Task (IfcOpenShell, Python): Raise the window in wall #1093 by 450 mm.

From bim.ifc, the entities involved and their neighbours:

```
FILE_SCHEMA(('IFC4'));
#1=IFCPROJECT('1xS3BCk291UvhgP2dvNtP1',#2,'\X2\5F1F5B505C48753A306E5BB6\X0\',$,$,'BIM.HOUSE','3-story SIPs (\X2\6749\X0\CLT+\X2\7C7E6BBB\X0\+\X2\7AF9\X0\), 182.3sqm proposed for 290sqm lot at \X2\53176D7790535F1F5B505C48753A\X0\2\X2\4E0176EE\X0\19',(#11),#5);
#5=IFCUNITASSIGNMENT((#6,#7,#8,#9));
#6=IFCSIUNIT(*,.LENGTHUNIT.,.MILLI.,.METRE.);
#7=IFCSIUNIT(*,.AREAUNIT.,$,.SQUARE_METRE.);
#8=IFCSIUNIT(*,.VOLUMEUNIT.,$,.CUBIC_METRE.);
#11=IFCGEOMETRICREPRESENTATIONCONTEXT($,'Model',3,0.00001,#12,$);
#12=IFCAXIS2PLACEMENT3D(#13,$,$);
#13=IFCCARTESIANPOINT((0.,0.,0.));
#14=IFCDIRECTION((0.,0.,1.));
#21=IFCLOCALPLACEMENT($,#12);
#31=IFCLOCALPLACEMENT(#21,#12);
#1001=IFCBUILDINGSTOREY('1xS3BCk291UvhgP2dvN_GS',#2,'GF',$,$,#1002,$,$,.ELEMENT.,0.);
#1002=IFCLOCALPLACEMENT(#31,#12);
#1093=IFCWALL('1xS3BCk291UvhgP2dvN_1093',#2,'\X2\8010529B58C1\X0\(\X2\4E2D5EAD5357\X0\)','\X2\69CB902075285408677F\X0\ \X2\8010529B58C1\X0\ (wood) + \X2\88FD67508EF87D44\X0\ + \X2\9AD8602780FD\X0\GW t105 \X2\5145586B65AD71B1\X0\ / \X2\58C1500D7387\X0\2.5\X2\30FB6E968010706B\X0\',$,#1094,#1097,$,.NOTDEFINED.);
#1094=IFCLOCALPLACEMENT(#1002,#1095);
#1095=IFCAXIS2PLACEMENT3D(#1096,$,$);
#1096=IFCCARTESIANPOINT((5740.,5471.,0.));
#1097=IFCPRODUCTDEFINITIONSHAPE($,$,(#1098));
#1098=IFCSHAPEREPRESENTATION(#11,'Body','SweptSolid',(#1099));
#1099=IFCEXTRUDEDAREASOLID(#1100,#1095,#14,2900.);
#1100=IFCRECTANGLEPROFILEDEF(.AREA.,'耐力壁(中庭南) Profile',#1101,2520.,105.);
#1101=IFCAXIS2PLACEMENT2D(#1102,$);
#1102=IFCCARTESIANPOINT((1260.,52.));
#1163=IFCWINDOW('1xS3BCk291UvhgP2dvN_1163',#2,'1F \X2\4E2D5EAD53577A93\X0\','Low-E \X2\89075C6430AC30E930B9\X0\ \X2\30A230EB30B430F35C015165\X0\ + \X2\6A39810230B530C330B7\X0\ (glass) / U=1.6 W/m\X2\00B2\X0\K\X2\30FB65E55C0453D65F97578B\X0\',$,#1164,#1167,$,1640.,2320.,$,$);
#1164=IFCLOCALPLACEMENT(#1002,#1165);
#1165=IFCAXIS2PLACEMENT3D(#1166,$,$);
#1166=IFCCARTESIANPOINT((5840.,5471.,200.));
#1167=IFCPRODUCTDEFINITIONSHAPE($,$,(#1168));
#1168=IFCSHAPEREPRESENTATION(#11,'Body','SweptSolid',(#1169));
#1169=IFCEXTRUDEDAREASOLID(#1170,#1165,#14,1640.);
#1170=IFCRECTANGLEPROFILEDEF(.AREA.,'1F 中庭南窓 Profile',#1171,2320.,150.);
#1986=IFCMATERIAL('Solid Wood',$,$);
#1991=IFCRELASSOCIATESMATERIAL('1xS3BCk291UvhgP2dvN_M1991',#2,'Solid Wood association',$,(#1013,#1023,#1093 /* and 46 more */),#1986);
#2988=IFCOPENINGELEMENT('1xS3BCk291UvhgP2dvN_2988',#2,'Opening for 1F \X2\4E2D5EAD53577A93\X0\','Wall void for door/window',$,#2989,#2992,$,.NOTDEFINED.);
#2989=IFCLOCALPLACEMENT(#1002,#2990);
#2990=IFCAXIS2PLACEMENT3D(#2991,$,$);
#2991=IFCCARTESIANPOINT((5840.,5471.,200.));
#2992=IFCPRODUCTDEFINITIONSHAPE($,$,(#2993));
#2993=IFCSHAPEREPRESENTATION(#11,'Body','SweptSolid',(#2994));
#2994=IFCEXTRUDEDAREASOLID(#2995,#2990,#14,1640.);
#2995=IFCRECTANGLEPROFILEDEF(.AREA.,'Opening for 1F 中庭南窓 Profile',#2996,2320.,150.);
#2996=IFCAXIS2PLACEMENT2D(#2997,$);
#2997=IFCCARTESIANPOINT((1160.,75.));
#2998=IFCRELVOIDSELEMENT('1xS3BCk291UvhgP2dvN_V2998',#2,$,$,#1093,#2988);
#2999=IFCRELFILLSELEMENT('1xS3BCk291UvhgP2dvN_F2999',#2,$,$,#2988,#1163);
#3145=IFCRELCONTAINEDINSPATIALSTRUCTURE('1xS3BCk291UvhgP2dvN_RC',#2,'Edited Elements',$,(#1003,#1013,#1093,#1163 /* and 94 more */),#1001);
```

```python
import numpy as np
import ifcopenshell
import ifcopenshell.api.geometry
import ifcopenshell.util.placement
import ifcopenshell.util.unit

model = ifcopenshell.open("bim.ifc")
unit_scale = ifcopenshell.util.unit.calculate_unit_scale(model)

window = model.by_id(1163)
opening = window.FillsVoids[0].RelatingOpeningElement
dz = 450.0

shift = np.array([0.0, 0.0, dz])
# The window is not placed relative to its opening, so move both.
for product in (opening, window):
    matrix = ifcopenshell.util.placement.get_local_placement(product.ObjectPlacement)
    matrix[:3, 3] += shift
    ifcopenshell.api.geometry.edit_object_placement(model, product=product, matrix=matrix, is_si=False)

print(f"moved by {dz * unit_scale:+.3f} m")

model.write("bim_edited.ifc")
```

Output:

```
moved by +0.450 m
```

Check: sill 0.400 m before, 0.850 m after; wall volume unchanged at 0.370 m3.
